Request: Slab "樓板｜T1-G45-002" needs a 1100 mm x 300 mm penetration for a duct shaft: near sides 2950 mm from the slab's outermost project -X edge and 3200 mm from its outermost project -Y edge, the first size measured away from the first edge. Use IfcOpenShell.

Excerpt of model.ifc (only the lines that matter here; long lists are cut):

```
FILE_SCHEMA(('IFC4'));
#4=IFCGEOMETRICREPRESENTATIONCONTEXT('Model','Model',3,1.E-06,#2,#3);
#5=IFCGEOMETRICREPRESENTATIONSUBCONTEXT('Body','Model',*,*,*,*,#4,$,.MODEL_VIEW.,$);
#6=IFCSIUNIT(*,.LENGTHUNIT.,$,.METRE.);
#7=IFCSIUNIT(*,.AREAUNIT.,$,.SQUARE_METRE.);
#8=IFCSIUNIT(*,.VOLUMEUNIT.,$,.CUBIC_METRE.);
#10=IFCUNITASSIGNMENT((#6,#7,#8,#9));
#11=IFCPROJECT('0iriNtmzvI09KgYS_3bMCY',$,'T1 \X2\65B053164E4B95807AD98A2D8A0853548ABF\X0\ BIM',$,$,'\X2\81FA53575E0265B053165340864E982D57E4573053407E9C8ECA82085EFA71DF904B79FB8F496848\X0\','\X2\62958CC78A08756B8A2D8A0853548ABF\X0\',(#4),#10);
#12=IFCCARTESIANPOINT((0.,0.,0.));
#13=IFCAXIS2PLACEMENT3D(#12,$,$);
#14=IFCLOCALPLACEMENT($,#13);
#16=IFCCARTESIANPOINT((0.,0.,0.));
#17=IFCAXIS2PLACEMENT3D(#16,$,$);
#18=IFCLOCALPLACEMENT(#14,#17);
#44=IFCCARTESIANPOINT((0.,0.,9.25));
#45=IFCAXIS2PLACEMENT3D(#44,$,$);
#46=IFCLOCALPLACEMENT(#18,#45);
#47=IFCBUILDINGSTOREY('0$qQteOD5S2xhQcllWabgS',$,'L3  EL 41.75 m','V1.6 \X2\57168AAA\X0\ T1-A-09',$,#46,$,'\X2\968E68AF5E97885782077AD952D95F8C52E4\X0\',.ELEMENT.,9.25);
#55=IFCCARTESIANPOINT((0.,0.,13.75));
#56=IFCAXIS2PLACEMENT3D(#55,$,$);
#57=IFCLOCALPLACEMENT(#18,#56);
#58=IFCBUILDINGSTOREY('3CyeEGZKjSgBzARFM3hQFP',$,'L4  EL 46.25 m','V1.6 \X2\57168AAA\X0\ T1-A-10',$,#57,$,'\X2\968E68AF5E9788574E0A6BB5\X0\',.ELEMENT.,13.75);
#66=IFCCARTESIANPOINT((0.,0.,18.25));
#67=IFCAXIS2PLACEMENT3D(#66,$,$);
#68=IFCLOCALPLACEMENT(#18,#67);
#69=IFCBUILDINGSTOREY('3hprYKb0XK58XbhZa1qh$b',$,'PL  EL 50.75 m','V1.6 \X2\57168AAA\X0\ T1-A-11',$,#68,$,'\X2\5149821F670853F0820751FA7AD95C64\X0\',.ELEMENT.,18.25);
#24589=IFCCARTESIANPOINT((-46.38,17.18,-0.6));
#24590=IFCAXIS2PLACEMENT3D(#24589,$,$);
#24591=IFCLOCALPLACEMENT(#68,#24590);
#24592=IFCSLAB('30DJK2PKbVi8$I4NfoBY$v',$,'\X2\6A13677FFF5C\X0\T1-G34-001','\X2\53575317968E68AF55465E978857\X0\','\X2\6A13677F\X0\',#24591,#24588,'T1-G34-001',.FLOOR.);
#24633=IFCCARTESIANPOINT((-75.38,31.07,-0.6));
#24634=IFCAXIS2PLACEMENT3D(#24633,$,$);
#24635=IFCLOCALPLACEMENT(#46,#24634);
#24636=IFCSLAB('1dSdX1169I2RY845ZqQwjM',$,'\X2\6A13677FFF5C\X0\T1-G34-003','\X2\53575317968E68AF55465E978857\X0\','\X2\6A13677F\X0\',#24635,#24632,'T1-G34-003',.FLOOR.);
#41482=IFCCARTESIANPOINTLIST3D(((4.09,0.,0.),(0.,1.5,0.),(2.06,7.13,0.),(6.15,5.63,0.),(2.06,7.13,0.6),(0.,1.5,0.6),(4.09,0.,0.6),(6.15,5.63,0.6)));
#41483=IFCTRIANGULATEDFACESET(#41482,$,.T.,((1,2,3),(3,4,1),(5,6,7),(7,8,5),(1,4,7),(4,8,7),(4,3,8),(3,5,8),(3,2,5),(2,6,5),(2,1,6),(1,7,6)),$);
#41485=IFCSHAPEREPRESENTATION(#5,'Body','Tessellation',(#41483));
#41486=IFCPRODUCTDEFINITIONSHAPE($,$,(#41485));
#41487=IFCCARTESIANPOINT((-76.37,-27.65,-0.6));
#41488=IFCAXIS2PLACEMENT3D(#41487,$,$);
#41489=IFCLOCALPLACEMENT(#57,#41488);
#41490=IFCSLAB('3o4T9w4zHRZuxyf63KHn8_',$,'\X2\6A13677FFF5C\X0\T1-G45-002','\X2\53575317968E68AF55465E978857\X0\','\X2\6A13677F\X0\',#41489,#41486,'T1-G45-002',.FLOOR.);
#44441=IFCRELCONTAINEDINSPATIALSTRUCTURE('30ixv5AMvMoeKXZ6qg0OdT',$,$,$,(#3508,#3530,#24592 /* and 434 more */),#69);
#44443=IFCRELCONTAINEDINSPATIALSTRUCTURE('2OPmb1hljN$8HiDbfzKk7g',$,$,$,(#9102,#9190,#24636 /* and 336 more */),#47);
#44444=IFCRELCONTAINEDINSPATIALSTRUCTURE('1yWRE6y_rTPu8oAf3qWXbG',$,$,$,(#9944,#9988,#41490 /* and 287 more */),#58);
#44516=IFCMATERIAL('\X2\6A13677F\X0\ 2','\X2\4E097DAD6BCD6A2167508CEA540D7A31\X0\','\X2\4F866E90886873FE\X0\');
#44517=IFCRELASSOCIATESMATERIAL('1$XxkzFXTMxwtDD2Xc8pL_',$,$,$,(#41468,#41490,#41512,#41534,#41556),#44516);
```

```python
import numpy as np
import ifcopenshell
import ifcopenshell.api.feature
import ifcopenshell.api.geometry
import ifcopenshell.api.root
import ifcopenshell.geom
import ifcopenshell.util.placement
import ifcopenshell.util.representation
import ifcopenshell.util.shape
import ifcopenshell.util.unit

model = ifcopenshell.open("model.ifc")
unit_scale = ifcopenshell.util.unit.calculate_unit_scale(model)
settings = ifcopenshell.geom.settings()


def volume(element):
    """Net volume in cubic metres, openings subtracted."""
    shape = ifcopenshell.geom.create_shape(settings, element)
    return ifcopenshell.util.shape.get_volume(shape.geometry)


slab = model.by_guid("3o4T9w4zHRZuxyf63KHn8_")
before = volume(slab)

# Extent in the slab's own axes, in metres. The edges named are its -X and -Y sides.
slab_shape = ifcopenshell.geom.create_shape(settings, slab)
vertices = ifcopenshell.util.shape.get_vertices(slab_shape.geometry)
x_min, y_min, bottom = vertices.min(axis=0)
top = vertices[:, 2].max()

opening = ifcopenshell.api.root.create_entity(model, ifc_class="IfcOpeningElement", name="Duct shaft opening", predefined_type="OPENING")
context = ifcopenshell.util.representation.get_context(model, "Model", "Body", "MODEL_VIEW")
width, depth = 1.1, 0.3
outline = [(0.0, 0.0), (width, 0.0), (width, depth), (0.0, depth), (0.0, 0.0)]
# Overshoot both faces by 50 mm so the cut is clean.
shape = ifcopenshell.api.geometry.add_slab_representation(
    model, context=context, depth=top - bottom + 0.1, polyline=outline
)
ifcopenshell.api.geometry.assign_representation(model, product=opening, representation=shape)

matrix = ifcopenshell.util.placement.get_local_placement(slab.ObjectPlacement)
matrix[:, 3] = matrix @ np.append(np.array([x_min + 2.95, y_min + 3.2, bottom - 0.05]) / unit_scale, 1.0)
ifcopenshell.api.geometry.edit_object_placement(model, product=opening, matrix=matrix, is_si=False)
ifcopenshell.api.feature.add_feature(model, feature=opening, element=slab)

after = volume(slab)

print(f"slab volume {before:.3f} -> {after:.3f} m3")

model.write("model_edited.ifc")
```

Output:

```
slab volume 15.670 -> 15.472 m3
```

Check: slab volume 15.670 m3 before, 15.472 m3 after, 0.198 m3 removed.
